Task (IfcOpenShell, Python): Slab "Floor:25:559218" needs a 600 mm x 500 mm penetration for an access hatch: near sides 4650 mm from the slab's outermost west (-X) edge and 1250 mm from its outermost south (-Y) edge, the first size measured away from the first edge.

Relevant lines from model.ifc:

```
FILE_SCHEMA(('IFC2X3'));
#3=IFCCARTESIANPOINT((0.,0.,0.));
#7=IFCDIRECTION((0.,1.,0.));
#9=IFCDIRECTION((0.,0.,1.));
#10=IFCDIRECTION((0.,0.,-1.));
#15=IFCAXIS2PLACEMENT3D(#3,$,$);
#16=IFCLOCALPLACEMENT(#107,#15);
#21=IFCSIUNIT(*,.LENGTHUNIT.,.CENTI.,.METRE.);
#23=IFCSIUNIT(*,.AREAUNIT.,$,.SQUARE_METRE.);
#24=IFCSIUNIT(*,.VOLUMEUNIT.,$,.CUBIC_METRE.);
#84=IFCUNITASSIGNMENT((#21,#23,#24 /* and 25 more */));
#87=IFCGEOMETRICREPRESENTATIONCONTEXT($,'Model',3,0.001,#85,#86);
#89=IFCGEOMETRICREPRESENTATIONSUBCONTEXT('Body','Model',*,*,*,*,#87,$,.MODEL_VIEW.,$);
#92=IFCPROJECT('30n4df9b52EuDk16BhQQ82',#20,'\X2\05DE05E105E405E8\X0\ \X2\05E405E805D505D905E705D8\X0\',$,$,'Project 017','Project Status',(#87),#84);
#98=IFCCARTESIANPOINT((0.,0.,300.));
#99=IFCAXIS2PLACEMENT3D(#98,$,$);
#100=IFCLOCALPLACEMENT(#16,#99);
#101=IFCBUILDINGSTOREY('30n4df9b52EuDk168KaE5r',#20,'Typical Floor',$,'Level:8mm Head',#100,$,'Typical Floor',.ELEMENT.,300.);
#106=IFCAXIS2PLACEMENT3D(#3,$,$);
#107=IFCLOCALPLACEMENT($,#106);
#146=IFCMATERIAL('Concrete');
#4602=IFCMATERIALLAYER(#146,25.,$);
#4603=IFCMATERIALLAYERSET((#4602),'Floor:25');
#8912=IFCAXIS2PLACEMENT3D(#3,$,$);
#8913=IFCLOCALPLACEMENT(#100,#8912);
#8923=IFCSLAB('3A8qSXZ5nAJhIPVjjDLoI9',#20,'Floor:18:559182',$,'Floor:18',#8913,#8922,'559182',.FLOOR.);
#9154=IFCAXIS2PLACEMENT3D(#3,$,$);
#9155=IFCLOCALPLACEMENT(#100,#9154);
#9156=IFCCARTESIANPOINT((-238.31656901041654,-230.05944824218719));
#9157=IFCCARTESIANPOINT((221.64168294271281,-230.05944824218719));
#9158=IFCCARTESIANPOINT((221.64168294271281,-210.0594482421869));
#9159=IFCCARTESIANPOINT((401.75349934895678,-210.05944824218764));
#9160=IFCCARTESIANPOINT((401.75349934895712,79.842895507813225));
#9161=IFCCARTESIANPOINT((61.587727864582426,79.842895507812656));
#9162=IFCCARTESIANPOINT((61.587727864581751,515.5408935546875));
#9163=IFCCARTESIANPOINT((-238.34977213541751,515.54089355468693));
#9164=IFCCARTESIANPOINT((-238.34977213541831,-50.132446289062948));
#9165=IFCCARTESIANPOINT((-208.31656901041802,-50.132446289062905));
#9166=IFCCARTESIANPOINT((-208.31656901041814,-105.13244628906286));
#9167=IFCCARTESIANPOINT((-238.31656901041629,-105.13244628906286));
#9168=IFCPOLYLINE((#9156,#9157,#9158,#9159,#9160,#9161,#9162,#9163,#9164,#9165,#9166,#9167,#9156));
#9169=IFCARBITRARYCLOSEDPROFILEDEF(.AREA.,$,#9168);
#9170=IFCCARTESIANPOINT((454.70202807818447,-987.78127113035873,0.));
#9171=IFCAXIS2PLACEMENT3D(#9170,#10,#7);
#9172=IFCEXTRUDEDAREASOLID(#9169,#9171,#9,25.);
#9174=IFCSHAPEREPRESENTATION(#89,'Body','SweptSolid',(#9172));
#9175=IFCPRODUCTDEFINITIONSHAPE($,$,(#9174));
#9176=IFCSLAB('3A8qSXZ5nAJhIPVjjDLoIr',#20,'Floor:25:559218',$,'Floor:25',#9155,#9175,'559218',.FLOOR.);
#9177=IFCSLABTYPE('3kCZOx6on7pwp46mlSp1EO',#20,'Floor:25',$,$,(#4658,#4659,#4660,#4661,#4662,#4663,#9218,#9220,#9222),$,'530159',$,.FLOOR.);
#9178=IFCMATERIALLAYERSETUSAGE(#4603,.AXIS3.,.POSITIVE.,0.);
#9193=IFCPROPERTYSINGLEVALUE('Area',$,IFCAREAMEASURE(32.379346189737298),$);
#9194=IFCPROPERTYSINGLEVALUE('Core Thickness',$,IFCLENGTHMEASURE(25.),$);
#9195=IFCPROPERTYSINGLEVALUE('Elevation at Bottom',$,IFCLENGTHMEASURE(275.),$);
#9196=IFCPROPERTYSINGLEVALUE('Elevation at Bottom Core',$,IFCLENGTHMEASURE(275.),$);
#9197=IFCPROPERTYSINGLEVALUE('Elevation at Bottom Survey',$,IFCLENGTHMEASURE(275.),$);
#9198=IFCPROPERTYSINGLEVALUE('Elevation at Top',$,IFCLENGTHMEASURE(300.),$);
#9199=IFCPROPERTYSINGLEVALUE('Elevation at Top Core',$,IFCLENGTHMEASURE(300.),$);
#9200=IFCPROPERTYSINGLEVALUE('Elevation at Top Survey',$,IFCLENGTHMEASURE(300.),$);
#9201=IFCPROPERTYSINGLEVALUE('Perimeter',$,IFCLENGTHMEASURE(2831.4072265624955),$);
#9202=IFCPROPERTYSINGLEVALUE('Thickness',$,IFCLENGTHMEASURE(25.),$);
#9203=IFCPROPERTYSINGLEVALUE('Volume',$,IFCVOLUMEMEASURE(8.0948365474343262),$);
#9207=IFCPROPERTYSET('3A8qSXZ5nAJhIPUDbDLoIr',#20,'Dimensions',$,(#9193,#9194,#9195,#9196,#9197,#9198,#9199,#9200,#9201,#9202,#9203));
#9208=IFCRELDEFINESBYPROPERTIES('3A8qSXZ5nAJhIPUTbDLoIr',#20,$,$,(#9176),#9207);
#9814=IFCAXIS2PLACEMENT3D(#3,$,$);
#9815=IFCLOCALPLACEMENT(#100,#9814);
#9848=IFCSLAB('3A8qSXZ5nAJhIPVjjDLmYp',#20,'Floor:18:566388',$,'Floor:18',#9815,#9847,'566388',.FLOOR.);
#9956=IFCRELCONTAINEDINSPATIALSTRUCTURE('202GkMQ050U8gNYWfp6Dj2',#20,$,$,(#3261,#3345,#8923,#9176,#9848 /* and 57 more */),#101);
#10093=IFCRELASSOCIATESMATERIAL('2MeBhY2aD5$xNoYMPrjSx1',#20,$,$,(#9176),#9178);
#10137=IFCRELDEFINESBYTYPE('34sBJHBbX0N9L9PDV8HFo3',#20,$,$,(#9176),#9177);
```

```python
import numpy as np
import ifcopenshell
import ifcopenshell.api.feature
import ifcopenshell.api.geometry
import ifcopenshell.api.pset
import ifcopenshell.api.root
import ifcopenshell.geom
import ifcopenshell.util.element
import ifcopenshell.util.placement
import ifcopenshell.util.representation
import ifcopenshell.util.shape
import ifcopenshell.util.unit

model = ifcopenshell.open("model.ifc")
unit_scale = ifcopenshell.util.unit.calculate_unit_scale(model)
area_scale = ifcopenshell.util.unit.calculate_unit_scale(model, "AREAUNIT")
volume_scale = ifcopenshell.util.unit.calculate_unit_scale(model, "VOLUMEUNIT")
settings = ifcopenshell.geom.settings()


def volume(element):
    """Net volume in cubic metres, openings subtracted."""
    shape = ifcopenshell.geom.create_shape(settings, element)
    return ifcopenshell.util.shape.get_volume(shape.geometry)


slab = model.by_id(9176)
before = volume(slab)

# Extent in the slab's own axes, in metres. The edges named are its -X and -Y sides.
slab_shape = ifcopenshell.geom.create_shape(settings, slab)
vertices = ifcopenshell.util.shape.get_vertices(slab_shape.geometry)
x_min, y_min, bottom = vertices.min(axis=0)
top = vertices[:, 2].max()

opening = ifcopenshell.api.root.create_entity(model, ifc_class="IfcOpeningElement", name="Access hatch opening")
context = ifcopenshell.util.representation.get_context(model, "Model", "Body", "MODEL_VIEW")
width, depth = 0.6, 0.5
outline = [(0.0, 0.0), (width, 0.0), (width, depth), (0.0, depth), (0.0, 0.0)]
# Overshoot both faces by 50 mm so the cut is clean.
shape = ifcopenshell.api.geometry.add_slab_representation(
    model, context=context, depth=top - bottom + 0.1, polyline=outline
)
ifcopenshell.api.geometry.assign_representation(model, product=opening, representation=shape)

matrix = ifcopenshell.util.placement.get_local_placement(slab.ObjectPlacement)
matrix[:, 3] = matrix @ np.append(np.array([x_min + 4.65, y_min + 1.25, bottom - 0.05]) / unit_scale, 1.0)
ifcopenshell.api.geometry.edit_object_placement(model, product=opening, matrix=matrix, is_si=False)
ifcopenshell.api.feature.add_feature(model, feature=opening, element=slab)

after = volume(slab)

# Update the slab's stored quantities.
pset = model.by_id(ifcopenshell.util.element.get_pset(slab, "Dimensions", should_inherit=False)["id"])
ifcopenshell.api.pset.edit_pset(model, pset=pset, properties={
    "Area": model.create_entity("IfcAreaMeasure", after / (top - bottom) / area_scale),
    "Volume": model.create_entity("IfcVolumeMeasure", after / volume_scale),
})

print(f"slab volume {before:.3f} -> {after:.3f} m3")

model.write("model_updated.ifc")
```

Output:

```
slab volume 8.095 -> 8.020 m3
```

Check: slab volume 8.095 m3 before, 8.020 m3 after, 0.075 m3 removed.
